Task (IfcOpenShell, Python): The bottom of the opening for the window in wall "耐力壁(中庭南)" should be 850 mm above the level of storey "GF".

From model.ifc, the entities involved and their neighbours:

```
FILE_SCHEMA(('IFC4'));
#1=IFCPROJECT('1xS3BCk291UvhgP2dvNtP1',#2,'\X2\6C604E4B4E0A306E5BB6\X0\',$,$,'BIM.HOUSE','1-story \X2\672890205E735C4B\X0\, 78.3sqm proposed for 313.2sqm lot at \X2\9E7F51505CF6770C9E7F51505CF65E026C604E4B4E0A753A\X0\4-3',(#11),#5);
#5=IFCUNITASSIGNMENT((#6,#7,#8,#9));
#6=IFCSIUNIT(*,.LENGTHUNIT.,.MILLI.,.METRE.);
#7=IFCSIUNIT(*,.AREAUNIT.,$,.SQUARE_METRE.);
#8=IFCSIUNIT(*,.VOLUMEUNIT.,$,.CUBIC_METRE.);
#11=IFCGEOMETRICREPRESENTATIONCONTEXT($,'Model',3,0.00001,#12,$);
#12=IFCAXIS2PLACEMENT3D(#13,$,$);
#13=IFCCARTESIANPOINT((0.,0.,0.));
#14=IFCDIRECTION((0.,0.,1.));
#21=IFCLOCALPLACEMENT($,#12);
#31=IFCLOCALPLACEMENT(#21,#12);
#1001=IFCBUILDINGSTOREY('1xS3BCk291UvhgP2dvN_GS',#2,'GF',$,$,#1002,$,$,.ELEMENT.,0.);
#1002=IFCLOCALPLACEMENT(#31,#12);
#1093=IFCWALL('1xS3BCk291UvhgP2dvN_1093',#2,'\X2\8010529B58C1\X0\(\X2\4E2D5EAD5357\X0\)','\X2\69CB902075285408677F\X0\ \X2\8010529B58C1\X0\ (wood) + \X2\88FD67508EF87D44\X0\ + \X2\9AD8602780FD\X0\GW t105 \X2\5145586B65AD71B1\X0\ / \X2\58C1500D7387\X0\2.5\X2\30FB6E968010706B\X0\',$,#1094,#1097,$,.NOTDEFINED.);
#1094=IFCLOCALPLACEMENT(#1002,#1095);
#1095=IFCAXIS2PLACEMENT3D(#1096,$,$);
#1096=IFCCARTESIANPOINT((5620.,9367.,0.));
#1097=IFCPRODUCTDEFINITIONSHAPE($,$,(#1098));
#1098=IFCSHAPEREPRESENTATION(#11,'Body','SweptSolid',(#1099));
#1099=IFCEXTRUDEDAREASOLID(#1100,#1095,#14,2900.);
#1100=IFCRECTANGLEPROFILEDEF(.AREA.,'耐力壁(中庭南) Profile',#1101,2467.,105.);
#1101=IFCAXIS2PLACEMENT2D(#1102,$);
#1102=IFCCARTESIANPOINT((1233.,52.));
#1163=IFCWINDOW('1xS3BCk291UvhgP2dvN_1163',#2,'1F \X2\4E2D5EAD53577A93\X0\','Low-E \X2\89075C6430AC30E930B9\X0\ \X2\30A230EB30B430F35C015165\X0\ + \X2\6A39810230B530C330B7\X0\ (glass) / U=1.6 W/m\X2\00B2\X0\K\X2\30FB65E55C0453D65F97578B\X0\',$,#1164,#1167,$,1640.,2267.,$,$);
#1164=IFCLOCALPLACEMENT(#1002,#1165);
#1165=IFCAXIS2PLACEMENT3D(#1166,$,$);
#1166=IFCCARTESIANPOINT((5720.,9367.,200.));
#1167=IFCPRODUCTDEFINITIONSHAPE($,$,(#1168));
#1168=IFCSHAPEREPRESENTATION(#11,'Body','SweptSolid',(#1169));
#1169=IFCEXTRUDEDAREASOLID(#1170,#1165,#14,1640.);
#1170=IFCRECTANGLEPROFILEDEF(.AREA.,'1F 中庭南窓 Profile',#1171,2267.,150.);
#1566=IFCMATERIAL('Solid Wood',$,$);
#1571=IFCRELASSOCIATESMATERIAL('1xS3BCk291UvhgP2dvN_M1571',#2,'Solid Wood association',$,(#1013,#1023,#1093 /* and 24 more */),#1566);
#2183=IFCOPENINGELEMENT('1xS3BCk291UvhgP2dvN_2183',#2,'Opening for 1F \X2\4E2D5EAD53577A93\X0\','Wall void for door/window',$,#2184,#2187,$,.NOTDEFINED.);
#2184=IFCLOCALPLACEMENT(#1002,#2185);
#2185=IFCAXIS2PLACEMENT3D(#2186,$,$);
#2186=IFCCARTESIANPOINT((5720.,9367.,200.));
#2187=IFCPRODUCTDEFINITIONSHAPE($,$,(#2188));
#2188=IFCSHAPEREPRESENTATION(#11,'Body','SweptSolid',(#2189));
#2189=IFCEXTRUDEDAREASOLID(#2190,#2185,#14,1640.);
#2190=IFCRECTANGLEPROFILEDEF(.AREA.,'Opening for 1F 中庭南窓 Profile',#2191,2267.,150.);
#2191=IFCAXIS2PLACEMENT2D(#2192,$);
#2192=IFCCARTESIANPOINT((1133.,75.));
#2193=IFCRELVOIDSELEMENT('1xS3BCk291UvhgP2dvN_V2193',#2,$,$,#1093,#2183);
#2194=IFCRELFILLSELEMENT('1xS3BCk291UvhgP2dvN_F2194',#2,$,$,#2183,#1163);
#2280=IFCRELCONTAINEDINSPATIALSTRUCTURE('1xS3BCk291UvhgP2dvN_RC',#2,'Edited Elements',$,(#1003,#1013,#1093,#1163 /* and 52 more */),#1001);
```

```python
import numpy as np
import ifcopenshell
import ifcopenshell.api.geometry
import ifcopenshell.geom
import ifcopenshell.util.element
import ifcopenshell.util.placement
import ifcopenshell.util.shape
import ifcopenshell.util.unit

model = ifcopenshell.open("model.ifc")
unit_scale = ifcopenshell.util.unit.calculate_unit_scale(model)

window = model.by_guid("1xS3BCk291UvhgP2dvN_1163")
opening = window.FillsVoids[0].RelatingOpeningElement
storey = ifcopenshell.util.element.get_container(window, ifc_class="IfcBuildingStorey")
level = ifcopenshell.util.placement.get_local_placement(storey.ObjectPlacement)[2, 3]

# The opening's origin need not be at the sill, so measure its lowest point.
shape = ifcopenshell.geom.create_shape(ifcopenshell.geom.settings(), opening)
bottom = ifcopenshell.util.shape.get_shape_bottom_elevation(shape, shape.geometry) / unit_scale
dz = level + 0.85 / unit_scale - bottom

shift = np.array([0.0, 0.0, dz])
# The window is not placed relative to its opening, so move both.
for product in (opening, window):
    matrix = ifcopenshell.util.placement.get_local_placement(product.ObjectPlacement)
    matrix[:3, 3] += shift
    ifcopenshell.api.geometry.edit_object_placement(model, product=product, matrix=matrix, is_si=False)

print(f"moved by {dz * unit_scale:+.3f} m")

model.write("model_edited.ifc")
```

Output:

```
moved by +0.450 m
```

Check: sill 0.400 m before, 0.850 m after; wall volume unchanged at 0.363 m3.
